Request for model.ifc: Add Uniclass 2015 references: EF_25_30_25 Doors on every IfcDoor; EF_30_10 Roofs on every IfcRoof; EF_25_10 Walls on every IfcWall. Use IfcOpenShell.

First a look at what the model holds.

```python
import ifcopenshell

model = ifcopenshell.open("model.ifc")
print(model.schema)
print("classifications:", [c.Name for c in model.by_type("IfcClassification")])
for ifc_class in ("IfcDoor", "IfcRoof", "IfcStair", "IfcWall", "IfcWindow"):
    print(ifc_class, len(model.by_type(ifc_class)))
```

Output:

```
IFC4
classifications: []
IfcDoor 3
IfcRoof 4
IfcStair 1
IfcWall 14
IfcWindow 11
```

```python
import ifcopenshell
import ifcopenshell.api.classification

model = ifcopenshell.open("model.ifc")

system = ifcopenshell.api.classification.add_classification(model, classification="Uniclass 2015")

codes = {
    "IfcDoor": ("EF_25_30_25", "Doors"),
    "IfcRoof": ("EF_30_10", "Roofs"),
    "IfcWall": ("EF_25_10", "Walls"),
}
for ifc_class, (code, name) in codes.items():
    products = model.by_type(ifc_class)
    ifcopenshell.api.classification.add_reference(
        model, products=products, classification=system, identification=code, name=name
    )
    print(code, len(products))

model.write("model_edited.ifc")
```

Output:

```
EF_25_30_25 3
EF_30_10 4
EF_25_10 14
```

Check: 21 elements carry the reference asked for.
